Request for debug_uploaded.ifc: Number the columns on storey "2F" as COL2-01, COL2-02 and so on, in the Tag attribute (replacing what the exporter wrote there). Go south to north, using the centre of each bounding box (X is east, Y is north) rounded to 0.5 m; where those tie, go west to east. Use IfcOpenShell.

First a look at what the model holds.

```python
import ifcopenshell
import ifcopenshell.util.element
import ifcopenshell.util.placement

model = ifcopenshell.open("debug_uploaded.ifc")
print(model.schema)
storey = next(s for s in model.by_type("IfcBuildingStorey") if s.Name == "2F")
columns = [e for e in ifcopenshell.util.element.get_decomposition(storey) if e.is_a("IfcColumn")]
for e in sorted(columns, key=lambda e: e.id()):
    origin = ifcopenshell.util.placement.get_local_placement(e.ObjectPlacement)[:3, 3]
    print(e.id(), e.Tag, e.Name, origin.round(2) + 0.0, sep=" | ")
```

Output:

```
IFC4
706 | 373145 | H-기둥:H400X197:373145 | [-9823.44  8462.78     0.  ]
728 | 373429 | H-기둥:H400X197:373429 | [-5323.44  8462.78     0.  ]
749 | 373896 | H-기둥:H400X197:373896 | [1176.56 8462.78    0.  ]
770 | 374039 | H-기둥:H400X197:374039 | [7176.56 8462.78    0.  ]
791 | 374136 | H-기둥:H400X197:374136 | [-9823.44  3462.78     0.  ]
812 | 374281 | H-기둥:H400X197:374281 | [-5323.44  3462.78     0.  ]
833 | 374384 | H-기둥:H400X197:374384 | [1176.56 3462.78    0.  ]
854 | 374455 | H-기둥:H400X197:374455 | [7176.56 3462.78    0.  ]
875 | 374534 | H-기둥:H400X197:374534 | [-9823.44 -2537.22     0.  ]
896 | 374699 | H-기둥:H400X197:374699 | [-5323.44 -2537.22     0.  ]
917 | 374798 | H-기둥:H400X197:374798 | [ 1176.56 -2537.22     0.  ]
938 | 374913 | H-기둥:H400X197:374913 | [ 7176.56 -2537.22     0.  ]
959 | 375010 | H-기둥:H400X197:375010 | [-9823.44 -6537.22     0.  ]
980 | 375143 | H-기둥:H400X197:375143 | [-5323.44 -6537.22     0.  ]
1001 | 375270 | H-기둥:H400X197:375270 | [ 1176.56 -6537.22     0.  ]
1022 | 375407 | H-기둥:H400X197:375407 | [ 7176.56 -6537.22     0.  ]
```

```python
import ifcopenshell
import ifcopenshell.geom
import ifcopenshell.util.element
import ifcopenshell.util.shape

model = ifcopenshell.open("debug_uploaded.ifc")
settings = ifcopenshell.geom.settings()
settings.set("use-world-coords", True)


def centre(element):
    shape = ifcopenshell.geom.create_shape(settings, element)
    return ifcopenshell.util.shape.get_bbox_centroid(shape.geometry)


storey = next(s for s in model.by_type("IfcBuildingStorey") if s.Name == "2F")
columns = [e for e in ifcopenshell.util.element.get_decomposition(storey) if e.is_a("IfcColumn")]

# Insertion points can sit at a corner or the storey origin, so sort by the geometry (in metres).
centres = {e: centre(e) for e in columns}
columns.sort(key=lambda e: (round(centres[e][1] / 0.5), centres[e][0]))

for i, e in enumerate(columns, start=1):
    number = f"COL2-{i:02d}"
    e.Tag = number
    print(e.id(), number)

model.write("debug_uploaded-out.ifc")
```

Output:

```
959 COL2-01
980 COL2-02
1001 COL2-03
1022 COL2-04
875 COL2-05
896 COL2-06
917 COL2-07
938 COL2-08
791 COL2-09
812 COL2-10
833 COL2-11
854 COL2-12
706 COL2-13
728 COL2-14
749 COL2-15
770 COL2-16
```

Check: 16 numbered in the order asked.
